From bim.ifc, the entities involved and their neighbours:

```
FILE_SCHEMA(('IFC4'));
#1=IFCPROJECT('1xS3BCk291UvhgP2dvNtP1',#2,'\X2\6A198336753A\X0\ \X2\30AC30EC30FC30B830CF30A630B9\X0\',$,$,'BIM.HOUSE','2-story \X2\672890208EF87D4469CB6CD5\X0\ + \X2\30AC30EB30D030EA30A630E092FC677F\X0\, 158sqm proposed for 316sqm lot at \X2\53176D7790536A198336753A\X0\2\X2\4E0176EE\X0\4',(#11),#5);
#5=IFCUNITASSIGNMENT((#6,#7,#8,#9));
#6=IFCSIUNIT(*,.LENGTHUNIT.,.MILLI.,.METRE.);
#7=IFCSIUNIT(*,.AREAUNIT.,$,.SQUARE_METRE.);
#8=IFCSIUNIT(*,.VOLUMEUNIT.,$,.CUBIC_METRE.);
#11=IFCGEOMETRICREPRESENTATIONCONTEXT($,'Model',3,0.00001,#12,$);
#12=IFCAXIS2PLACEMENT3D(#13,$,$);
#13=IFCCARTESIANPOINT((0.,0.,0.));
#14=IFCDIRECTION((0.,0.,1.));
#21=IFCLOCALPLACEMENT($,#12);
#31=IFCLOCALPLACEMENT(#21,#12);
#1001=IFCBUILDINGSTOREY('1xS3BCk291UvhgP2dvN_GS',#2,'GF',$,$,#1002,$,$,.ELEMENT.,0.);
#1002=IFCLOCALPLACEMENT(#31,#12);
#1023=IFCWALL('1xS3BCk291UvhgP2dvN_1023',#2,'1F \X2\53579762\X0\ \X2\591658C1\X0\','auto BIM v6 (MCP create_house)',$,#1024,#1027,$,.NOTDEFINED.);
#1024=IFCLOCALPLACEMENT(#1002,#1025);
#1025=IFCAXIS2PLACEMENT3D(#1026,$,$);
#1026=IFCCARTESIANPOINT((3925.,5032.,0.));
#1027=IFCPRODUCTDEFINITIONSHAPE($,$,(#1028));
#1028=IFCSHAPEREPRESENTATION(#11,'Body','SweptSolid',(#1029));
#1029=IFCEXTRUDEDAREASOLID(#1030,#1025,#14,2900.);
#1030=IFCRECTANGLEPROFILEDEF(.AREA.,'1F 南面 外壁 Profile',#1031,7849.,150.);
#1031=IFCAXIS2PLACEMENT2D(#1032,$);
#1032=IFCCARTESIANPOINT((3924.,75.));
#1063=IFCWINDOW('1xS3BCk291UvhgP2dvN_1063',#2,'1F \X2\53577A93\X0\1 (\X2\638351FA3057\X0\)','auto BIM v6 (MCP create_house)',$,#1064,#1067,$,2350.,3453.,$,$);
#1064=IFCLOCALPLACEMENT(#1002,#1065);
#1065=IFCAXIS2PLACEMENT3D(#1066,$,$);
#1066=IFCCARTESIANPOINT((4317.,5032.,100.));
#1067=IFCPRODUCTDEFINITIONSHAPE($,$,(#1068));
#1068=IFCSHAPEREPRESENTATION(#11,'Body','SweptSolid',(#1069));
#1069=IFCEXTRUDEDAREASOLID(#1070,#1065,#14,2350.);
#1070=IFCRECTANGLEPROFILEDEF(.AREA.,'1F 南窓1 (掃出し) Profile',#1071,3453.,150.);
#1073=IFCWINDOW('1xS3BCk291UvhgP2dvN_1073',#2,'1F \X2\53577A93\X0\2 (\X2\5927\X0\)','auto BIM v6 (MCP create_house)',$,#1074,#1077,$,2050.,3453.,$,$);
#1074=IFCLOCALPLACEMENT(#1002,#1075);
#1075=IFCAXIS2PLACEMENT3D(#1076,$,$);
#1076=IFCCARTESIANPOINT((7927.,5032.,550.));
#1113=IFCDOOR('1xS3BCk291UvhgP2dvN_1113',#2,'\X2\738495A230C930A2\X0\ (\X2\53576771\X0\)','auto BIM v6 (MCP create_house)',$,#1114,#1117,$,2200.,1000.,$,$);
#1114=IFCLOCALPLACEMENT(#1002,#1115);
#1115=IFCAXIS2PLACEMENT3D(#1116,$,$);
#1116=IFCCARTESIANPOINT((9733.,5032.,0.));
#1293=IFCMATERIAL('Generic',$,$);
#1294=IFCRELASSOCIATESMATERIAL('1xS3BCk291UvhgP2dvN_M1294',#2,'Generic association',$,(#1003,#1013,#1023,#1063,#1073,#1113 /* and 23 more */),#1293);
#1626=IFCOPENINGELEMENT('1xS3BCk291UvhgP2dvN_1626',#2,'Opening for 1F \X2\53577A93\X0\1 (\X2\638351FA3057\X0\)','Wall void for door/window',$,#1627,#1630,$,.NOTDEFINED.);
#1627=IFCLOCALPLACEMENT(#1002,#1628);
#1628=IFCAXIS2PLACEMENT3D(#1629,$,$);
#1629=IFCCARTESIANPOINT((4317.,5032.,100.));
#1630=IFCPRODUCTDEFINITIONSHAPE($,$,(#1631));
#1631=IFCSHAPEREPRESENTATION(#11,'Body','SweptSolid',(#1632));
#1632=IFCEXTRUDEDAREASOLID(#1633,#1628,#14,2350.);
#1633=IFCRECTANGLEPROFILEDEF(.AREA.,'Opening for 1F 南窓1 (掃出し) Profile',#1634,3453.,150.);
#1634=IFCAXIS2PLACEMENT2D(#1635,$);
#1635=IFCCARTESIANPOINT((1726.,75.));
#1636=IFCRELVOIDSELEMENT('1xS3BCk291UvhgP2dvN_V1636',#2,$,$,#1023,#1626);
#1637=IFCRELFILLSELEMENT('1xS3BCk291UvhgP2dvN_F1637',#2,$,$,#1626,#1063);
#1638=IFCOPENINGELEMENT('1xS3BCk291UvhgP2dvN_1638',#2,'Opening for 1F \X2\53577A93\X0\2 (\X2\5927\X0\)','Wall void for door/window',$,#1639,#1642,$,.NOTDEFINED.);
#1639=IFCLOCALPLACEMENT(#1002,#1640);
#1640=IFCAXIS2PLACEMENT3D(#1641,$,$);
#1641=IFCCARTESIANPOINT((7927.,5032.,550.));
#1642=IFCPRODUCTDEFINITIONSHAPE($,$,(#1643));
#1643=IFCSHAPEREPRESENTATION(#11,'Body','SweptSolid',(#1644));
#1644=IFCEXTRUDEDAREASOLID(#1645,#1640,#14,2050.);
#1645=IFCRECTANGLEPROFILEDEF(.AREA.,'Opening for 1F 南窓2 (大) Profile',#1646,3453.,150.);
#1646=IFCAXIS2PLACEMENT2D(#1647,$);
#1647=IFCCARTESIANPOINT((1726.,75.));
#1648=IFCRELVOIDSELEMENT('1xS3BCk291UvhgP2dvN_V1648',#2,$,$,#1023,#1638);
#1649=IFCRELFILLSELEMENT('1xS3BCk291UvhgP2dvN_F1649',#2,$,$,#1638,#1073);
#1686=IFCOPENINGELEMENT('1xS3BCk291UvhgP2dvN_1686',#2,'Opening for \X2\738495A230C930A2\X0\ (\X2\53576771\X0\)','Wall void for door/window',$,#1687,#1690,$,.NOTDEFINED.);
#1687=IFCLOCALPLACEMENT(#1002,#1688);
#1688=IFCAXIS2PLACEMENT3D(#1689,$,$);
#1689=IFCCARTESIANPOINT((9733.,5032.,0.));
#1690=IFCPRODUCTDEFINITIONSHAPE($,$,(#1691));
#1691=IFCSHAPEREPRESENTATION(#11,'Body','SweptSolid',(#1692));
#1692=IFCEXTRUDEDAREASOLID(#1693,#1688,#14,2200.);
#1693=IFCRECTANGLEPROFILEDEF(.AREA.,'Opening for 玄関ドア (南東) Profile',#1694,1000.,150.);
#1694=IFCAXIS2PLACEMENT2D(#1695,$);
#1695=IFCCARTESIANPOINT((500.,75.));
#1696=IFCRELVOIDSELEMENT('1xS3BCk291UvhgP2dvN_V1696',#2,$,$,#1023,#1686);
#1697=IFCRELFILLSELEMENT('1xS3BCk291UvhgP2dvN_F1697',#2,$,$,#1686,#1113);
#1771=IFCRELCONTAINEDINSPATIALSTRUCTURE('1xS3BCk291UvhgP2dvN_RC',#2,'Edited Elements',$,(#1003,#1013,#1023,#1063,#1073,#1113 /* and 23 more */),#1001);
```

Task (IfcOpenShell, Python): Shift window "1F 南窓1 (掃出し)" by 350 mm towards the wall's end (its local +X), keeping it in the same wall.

```python
import ifcopenshell
import ifcopenshell.api.geometry
import ifcopenshell.util.placement
import ifcopenshell.util.unit

model = ifcopenshell.open("bim.ifc")
unit_scale = ifcopenshell.util.unit.calculate_unit_scale(model)

window = model.by_guid("1xS3BCk291UvhgP2dvN_1063")
opening = window.FillsVoids[0].RelatingOpeningElement
wall = opening.VoidsElements[0].RelatingBuildingElement

wall_matrix = ifcopenshell.util.placement.get_local_placement(wall.ObjectPlacement)
shift = wall_matrix[:3, 0] * 0.35 / unit_scale
before = ifcopenshell.util.placement.get_local_placement(window.ObjectPlacement)[:3, 3].copy()

# The window is not placed relative to its opening, so move both.
for product in (opening, window):
    matrix = ifcopenshell.util.placement.get_local_placement(product.ObjectPlacement)
    matrix[:3, 3] += shift
    ifcopenshell.api.geometry.edit_object_placement(model, product=product, matrix=matrix, is_si=False)

after = ifcopenshell.util.placement.get_local_placement(window.ObjectPlacement)[:3, 3]
print("window moved by", (after - before).round(3) + 0.0)

model.write("bim_updated.ifc")
```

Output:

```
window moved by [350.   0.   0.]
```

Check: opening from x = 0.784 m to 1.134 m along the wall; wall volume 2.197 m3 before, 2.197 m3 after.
